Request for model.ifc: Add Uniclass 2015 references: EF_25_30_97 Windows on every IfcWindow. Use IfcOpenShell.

First a look at what the model holds.

```python
import ifcopenshell

model = ifcopenshell.open("model.ifc")
print(model.schema)
print("classifications:", [c.Name for c in model.by_type("IfcClassification")])
for ifc_class in ("IfcDoor", "IfcRoof", "IfcStair", "IfcWall", "IfcWindow"):
    print(ifc_class, len(model.by_type(ifc_class)))
```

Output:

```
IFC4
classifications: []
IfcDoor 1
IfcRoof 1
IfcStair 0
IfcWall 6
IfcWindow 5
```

```python
import ifcopenshell
import ifcopenshell.api.classification

model = ifcopenshell.open("model.ifc")

system = ifcopenshell.api.classification.add_classification(model, classification="Uniclass 2015")

codes = {
    "IfcWindow": ("EF_25_30_97", "Windows"),
}
for ifc_class, (code, name) in codes.items():
    products = model.by_type(ifc_class)
    ifcopenshell.api.classification.add_reference(
        model, products=products, classification=system, identification=code, name=name
    )
    print(code, len(products))

model.write("model_edited.ifc")
```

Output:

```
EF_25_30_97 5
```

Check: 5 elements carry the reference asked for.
